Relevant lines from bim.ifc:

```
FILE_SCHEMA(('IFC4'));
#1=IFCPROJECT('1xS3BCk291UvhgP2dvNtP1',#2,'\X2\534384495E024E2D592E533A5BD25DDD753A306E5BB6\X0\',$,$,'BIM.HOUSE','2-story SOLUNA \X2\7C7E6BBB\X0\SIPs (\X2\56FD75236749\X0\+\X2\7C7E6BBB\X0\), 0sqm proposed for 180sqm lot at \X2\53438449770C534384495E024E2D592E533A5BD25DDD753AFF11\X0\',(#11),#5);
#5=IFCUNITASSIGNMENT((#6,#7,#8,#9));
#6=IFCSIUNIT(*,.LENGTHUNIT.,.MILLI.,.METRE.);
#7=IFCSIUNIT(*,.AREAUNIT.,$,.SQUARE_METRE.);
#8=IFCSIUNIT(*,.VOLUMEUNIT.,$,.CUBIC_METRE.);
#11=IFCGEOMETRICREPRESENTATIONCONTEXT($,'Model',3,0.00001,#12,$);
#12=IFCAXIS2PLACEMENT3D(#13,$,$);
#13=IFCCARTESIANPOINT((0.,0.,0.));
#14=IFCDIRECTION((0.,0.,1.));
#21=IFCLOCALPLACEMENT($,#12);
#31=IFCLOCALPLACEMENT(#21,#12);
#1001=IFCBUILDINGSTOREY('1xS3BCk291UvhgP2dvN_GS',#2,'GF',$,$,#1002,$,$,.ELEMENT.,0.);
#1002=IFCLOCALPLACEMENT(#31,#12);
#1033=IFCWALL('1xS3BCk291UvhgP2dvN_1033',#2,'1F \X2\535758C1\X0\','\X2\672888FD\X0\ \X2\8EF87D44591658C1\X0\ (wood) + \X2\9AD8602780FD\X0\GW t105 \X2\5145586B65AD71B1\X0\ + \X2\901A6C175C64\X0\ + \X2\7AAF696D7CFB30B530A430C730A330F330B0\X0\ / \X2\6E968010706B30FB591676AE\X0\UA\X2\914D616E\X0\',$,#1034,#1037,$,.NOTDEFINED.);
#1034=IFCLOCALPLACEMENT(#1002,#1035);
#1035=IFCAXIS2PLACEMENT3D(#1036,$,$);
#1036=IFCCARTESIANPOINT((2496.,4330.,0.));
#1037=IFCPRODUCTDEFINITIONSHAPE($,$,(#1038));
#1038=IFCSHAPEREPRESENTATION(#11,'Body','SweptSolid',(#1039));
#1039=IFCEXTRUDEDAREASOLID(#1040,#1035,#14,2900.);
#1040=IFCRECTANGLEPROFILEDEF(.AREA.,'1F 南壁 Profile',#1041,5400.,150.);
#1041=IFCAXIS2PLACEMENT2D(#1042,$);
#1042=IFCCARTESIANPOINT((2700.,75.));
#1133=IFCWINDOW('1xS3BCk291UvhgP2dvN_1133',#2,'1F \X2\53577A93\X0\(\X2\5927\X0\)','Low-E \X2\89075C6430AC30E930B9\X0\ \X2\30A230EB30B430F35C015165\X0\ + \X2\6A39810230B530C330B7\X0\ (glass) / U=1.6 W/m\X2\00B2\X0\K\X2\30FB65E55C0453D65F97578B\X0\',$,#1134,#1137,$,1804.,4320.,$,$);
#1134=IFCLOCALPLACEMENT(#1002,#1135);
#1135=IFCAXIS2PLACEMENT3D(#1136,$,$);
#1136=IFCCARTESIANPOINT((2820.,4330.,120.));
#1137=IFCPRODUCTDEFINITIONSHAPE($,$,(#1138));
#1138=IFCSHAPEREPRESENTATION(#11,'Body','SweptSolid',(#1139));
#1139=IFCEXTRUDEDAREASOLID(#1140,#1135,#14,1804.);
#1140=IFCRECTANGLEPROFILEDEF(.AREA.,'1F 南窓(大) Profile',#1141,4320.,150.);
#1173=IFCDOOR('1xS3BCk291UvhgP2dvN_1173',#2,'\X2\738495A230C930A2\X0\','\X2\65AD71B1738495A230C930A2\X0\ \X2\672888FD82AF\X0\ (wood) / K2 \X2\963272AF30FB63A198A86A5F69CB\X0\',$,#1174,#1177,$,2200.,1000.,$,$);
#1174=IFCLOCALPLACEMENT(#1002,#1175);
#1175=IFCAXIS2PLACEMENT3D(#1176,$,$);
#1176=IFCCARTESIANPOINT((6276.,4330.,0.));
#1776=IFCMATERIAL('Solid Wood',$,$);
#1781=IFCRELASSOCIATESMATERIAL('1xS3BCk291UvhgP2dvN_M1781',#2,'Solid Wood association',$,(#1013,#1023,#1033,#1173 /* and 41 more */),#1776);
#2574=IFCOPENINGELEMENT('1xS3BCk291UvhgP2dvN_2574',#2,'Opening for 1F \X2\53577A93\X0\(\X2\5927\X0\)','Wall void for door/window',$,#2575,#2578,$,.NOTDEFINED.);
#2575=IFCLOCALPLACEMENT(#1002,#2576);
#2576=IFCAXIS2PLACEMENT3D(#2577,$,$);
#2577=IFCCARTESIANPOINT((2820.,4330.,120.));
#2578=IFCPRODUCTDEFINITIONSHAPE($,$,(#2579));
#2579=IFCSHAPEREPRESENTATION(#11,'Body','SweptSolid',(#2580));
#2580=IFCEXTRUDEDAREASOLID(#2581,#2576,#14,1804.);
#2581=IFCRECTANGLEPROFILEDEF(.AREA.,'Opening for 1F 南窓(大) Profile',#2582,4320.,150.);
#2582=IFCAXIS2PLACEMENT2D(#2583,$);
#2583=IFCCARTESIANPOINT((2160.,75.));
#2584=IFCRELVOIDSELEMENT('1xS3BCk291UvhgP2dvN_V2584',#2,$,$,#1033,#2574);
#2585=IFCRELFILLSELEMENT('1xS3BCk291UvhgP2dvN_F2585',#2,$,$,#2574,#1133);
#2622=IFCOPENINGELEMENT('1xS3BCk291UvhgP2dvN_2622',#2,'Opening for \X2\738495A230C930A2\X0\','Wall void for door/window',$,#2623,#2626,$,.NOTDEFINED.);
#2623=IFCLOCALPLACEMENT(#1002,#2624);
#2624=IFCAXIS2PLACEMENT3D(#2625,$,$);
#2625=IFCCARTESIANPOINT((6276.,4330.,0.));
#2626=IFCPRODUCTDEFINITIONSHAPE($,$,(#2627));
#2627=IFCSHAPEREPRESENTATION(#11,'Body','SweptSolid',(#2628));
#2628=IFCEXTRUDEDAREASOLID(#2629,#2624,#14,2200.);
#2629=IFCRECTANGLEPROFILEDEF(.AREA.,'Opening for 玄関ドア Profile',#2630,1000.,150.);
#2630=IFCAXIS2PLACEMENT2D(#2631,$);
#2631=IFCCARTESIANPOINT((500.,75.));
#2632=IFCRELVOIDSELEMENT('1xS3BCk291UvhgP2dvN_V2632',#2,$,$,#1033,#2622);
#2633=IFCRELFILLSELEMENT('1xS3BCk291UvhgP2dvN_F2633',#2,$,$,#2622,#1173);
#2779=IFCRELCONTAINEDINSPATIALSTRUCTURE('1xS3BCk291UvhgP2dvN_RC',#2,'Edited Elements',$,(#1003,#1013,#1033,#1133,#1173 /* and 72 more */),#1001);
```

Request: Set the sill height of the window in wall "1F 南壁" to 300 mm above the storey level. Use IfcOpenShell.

```python
import numpy as np
import ifcopenshell
import ifcopenshell.api.geometry
import ifcopenshell.geom
import ifcopenshell.util.element
import ifcopenshell.util.placement
import ifcopenshell.util.shape
import ifcopenshell.util.unit

model = ifcopenshell.open("bim.ifc")
unit_scale = ifcopenshell.util.unit.calculate_unit_scale(model)

window = model.by_guid("1xS3BCk291UvhgP2dvN_1133")
opening = window.FillsVoids[0].RelatingOpeningElement
storey = ifcopenshell.util.element.get_container(window, ifc_class="IfcBuildingStorey")
level = ifcopenshell.util.placement.get_local_placement(storey.ObjectPlacement)[2, 3]

# The opening's origin need not be at the sill, so measure its lowest point.
shape = ifcopenshell.geom.create_shape(ifcopenshell.geom.settings(), opening)
bottom = ifcopenshell.util.shape.get_shape_bottom_elevation(shape, shape.geometry) / unit_scale
dz = level + 300.0 - bottom

shift = np.array([0.0, 0.0, dz])
# The window is not placed relative to its opening, so move both.
for product in (opening, window):
    matrix = ifcopenshell.util.placement.get_local_placement(product.ObjectPlacement)
    matrix[:3, 3] += shift
    ifcopenshell.api.geometry.edit_object_placement(model, product=product, matrix=matrix, is_si=False)

print(f"moved by {dz * unit_scale:+.3f} m")

model.write("bim-out.ifc")
```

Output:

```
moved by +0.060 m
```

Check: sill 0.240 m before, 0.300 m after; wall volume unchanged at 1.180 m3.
